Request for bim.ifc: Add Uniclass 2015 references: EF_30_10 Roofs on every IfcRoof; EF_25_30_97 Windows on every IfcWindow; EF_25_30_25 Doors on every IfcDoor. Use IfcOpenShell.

First a look at what the model holds.

```python
import ifcopenshell

model = ifcopenshell.open("bim.ifc")
print(model.schema)
print("classifications:", [c.Name for c in model.by_type("IfcClassification")])
for ifc_class in ("IfcDoor", "IfcRoof", "IfcStair", "IfcWall", "IfcWindow"):
    print(ifc_class, len(model.by_type(ifc_class)))
```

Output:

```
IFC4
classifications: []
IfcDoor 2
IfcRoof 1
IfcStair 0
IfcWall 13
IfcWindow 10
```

```python
import ifcopenshell
import ifcopenshell.api.classification

model = ifcopenshell.open("bim.ifc")

system = ifcopenshell.api.classification.add_classification(model, classification="Uniclass 2015")

codes = {
    "IfcRoof": ("EF_30_10", "Roofs"),
    "IfcWindow": ("EF_25_30_97", "Windows"),
    "IfcDoor": ("EF_25_30_25", "Doors"),
}
for ifc_class, (code, name) in codes.items():
    products = model.by_type(ifc_class)
    ifcopenshell.api.classification.add_reference(
        model, products=products, classification=system, identification=code, name=name
    )
    print(code, len(products))

model.write("bim-out.ifc")
```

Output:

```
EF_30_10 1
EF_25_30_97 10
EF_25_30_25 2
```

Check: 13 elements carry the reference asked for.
